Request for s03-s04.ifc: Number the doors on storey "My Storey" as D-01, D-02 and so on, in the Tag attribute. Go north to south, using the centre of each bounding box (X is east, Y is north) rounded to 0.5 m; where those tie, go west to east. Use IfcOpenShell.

First a look at what the model holds.

```python
import ifcopenshell
import ifcopenshell.util.element
import ifcopenshell.util.placement

model = ifcopenshell.open("s03-s04.ifc")
print(model.schema)
storey = next(s for s in model.by_type("IfcBuildingStorey") if s.Name == "My Storey")
doors = [e for e in ifcopenshell.util.element.get_decomposition(storey) if e.is_a("IfcDoor")]
for e in sorted(doors, key=lambda e: e.id()):
    origin = ifcopenshell.util.placement.get_local_placement(e.ObjectPlacement)[:3, 3]
    print(e.id(), e.Tag, e.Name, origin.round(2) + 0.0, sep=" | ")
```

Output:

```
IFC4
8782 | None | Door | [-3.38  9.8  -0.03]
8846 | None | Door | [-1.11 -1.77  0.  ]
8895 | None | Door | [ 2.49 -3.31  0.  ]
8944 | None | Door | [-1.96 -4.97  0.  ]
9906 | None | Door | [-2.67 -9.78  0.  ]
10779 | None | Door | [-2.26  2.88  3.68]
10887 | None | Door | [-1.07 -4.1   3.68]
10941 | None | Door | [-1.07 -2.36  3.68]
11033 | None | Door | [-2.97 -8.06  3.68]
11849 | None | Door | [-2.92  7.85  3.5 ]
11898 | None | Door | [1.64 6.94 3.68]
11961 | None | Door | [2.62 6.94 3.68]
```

```python
import ifcopenshell
import ifcopenshell.geom
import ifcopenshell.util.element
import ifcopenshell.util.shape

model = ifcopenshell.open("s03-s04.ifc")
settings = ifcopenshell.geom.settings()
settings.set("use-world-coords", True)


def centre(element):
    shape = ifcopenshell.geom.create_shape(settings, element)
    return ifcopenshell.util.shape.get_bbox_centroid(shape.geometry)


storey = next(s for s in model.by_type("IfcBuildingStorey") if s.Name == "My Storey")
doors = [e for e in ifcopenshell.util.element.get_decomposition(storey) if e.is_a("IfcDoor")]

# Insertion points can sit at a corner or the storey origin, so sort by the geometry (in metres).
centres = {e: centre(e) for e in doors}
doors.sort(key=lambda e: (-round(centres[e][1] / 0.5), centres[e][0]))

for i, e in enumerate(doors, start=1):
    number = f"D-{i:02d}"
    e.Tag = number
    print(e.id(), number)

model.write("s03-s04-out.ifc")
```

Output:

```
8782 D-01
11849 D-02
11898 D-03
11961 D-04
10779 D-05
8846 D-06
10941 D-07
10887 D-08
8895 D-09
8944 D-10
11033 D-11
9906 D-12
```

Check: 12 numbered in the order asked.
